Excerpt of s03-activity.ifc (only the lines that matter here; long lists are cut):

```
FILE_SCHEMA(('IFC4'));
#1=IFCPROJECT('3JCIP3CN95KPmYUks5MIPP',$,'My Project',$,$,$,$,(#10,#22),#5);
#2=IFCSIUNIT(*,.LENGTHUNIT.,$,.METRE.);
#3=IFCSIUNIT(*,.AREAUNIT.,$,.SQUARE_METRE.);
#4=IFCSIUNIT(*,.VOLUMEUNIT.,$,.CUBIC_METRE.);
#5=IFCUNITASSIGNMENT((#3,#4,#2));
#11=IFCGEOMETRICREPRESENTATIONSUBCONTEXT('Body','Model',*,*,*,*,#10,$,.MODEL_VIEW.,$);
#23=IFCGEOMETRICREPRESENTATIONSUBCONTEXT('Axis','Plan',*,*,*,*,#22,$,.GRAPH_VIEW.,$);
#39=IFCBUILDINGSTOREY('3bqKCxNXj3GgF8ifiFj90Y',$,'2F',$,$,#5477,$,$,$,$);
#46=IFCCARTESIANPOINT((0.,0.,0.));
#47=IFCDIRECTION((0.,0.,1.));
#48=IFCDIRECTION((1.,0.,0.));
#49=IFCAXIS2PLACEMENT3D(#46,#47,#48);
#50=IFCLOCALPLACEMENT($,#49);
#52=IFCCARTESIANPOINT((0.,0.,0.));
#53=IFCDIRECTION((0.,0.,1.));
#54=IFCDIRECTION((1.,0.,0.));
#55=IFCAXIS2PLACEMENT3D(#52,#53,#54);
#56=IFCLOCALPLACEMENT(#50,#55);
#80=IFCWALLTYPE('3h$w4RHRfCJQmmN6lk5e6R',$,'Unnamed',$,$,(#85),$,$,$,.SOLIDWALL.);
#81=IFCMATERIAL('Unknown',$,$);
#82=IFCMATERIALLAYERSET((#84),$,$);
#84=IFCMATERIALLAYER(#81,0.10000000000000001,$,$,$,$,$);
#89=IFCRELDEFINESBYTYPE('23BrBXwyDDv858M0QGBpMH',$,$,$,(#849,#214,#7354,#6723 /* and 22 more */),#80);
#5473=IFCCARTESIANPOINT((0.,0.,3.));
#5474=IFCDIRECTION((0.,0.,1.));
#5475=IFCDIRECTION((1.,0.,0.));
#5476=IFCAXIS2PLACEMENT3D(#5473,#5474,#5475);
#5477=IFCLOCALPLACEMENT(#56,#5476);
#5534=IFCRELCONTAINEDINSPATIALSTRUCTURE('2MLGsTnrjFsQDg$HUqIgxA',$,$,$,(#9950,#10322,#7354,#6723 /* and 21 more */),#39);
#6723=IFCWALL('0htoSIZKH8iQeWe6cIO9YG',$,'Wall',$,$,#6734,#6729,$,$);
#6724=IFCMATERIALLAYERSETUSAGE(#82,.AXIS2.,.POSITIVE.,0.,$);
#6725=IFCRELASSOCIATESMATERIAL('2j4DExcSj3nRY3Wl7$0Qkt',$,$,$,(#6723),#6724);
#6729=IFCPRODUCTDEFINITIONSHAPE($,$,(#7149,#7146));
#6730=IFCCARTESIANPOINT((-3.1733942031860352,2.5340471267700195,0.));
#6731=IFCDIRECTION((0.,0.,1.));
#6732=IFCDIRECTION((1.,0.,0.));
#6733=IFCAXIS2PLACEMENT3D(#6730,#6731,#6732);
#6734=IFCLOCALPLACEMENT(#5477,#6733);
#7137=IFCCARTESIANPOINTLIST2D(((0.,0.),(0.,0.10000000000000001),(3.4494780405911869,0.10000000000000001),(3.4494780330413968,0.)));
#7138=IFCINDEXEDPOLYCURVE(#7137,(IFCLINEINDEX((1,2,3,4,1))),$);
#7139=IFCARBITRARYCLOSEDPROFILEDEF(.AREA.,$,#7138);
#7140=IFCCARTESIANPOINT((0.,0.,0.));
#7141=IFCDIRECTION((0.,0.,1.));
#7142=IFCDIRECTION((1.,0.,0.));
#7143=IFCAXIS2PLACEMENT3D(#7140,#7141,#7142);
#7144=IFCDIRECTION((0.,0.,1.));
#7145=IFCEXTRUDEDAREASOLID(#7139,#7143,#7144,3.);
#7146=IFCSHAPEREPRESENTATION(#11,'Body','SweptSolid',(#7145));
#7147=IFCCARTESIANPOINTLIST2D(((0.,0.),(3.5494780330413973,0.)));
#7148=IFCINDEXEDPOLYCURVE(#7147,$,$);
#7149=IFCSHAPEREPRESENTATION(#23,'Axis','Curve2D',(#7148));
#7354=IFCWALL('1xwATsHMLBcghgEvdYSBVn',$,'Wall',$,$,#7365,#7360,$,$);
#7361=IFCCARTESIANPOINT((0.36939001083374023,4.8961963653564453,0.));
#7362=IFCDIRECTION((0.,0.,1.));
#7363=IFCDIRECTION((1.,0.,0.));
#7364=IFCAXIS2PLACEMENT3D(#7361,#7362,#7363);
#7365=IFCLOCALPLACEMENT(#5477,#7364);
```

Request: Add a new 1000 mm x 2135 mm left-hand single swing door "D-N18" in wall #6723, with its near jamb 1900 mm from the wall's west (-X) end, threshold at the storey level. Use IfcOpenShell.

```python
import numpy as np
import ifcopenshell
import ifcopenshell.api.feature
import ifcopenshell.api.geometry
import ifcopenshell.api.root
import ifcopenshell.api.spatial
import ifcopenshell.geom
import ifcopenshell.util.element
import ifcopenshell.util.placement
import ifcopenshell.util.representation
import ifcopenshell.util.shape
import ifcopenshell.util.unit

model = ifcopenshell.open("s03-activity.ifc")
unit_scale = ifcopenshell.util.unit.calculate_unit_scale(model)
settings = ifcopenshell.geom.settings()


def volume(element):
    """Net volume in cubic metres, openings subtracted."""
    shape = ifcopenshell.geom.create_shape(settings, element)
    return ifcopenshell.util.shape.get_volume(shape.geometry)


wall = model.by_guid("0htoSIZKH8iQeWe6cIO9YG")
storey = ifcopenshell.util.element.get_container(wall, ifc_class="IfcBuildingStorey")
context = ifcopenshell.util.representation.get_context(model, "Model", "Body", "MODEL_VIEW")
before = volume(wall)

width, height, from_end, sill = 1, 2.135, 1.9, 0.0  # metres

# The wall runs along its own X axis, and the end named is its -X end.
wall_shape = ifcopenshell.geom.create_shape(settings, wall)
x, y, z = ifcopenshell.util.shape.get_vertices(wall_shape.geometry).T
start = x.min() + from_end
face, thickness = float(y.min()), float(y.max() - y.min())
wall_matrix = ifcopenshell.util.placement.get_local_placement(wall.ObjectPlacement)
level = ifcopenshell.util.placement.get_local_placement(storey.ObjectPlacement)[2, 3]


def in_wall(x, y):
    """Placement at x, y metres in the wall's axes, at sill height."""
    matrix = wall_matrix.copy()
    matrix[:, 3] = wall_matrix @ np.array([x / unit_scale, y / unit_scale, 0.0, 1.0])
    matrix[2, 3] = level + sill / unit_scale
    return matrix


# Opening: a box that overshoots both wall faces by 50 mm.
opening = ifcopenshell.api.root.create_entity(model, ifc_class="IfcOpeningElement", predefined_type="OPENING")
box = ifcopenshell.api.geometry.add_wall_representation(
    model, context=context, length=width, height=height, thickness=thickness + 0.1
)
ifcopenshell.api.geometry.assign_representation(model, product=opening, representation=box)
ifcopenshell.api.geometry.edit_object_placement(model, product=opening, matrix=in_wall(start, face - 0.05), is_si=False)
ifcopenshell.api.feature.add_feature(model, feature=opening, element=wall)

door = ifcopenshell.api.root.create_entity(model, ifc_class="IfcDoor", name="D-N18", predefined_type="DOOR")
door.OverallWidth, door.OverallHeight = width / unit_scale, height / unit_scale
door.OperationType = "SINGLE_SWING_LEFT"
body = ifcopenshell.api.geometry.add_door_representation(
    model,
    context=context,
    overall_width=door.OverallWidth,
    overall_height=door.OverallHeight,
    operation_type="SINGLE_SWING_LEFT",
    lining_properties={"LiningDepth": thickness / unit_scale, "ThresholdDepth": thickness / unit_scale},
)
ifcopenshell.api.geometry.assign_representation(model, product=door, representation=body)
ifcopenshell.api.spatial.assign_container(model, products=[door], relating_structure=storey)
ifcopenshell.api.feature.add_filling(model, opening=opening, element=door)

# The lining spans the wall, so the door starts at the wall face.
ifcopenshell.api.geometry.edit_object_placement(model, product=door, matrix=in_wall(start, face), is_si=False)

after = volume(wall)

print(f"wall volume {before:.3f} -> {after:.3f} m3")

model.write("s03-activity_updated.ifc")
```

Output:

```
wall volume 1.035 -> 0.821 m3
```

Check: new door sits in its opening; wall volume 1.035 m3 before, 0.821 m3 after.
